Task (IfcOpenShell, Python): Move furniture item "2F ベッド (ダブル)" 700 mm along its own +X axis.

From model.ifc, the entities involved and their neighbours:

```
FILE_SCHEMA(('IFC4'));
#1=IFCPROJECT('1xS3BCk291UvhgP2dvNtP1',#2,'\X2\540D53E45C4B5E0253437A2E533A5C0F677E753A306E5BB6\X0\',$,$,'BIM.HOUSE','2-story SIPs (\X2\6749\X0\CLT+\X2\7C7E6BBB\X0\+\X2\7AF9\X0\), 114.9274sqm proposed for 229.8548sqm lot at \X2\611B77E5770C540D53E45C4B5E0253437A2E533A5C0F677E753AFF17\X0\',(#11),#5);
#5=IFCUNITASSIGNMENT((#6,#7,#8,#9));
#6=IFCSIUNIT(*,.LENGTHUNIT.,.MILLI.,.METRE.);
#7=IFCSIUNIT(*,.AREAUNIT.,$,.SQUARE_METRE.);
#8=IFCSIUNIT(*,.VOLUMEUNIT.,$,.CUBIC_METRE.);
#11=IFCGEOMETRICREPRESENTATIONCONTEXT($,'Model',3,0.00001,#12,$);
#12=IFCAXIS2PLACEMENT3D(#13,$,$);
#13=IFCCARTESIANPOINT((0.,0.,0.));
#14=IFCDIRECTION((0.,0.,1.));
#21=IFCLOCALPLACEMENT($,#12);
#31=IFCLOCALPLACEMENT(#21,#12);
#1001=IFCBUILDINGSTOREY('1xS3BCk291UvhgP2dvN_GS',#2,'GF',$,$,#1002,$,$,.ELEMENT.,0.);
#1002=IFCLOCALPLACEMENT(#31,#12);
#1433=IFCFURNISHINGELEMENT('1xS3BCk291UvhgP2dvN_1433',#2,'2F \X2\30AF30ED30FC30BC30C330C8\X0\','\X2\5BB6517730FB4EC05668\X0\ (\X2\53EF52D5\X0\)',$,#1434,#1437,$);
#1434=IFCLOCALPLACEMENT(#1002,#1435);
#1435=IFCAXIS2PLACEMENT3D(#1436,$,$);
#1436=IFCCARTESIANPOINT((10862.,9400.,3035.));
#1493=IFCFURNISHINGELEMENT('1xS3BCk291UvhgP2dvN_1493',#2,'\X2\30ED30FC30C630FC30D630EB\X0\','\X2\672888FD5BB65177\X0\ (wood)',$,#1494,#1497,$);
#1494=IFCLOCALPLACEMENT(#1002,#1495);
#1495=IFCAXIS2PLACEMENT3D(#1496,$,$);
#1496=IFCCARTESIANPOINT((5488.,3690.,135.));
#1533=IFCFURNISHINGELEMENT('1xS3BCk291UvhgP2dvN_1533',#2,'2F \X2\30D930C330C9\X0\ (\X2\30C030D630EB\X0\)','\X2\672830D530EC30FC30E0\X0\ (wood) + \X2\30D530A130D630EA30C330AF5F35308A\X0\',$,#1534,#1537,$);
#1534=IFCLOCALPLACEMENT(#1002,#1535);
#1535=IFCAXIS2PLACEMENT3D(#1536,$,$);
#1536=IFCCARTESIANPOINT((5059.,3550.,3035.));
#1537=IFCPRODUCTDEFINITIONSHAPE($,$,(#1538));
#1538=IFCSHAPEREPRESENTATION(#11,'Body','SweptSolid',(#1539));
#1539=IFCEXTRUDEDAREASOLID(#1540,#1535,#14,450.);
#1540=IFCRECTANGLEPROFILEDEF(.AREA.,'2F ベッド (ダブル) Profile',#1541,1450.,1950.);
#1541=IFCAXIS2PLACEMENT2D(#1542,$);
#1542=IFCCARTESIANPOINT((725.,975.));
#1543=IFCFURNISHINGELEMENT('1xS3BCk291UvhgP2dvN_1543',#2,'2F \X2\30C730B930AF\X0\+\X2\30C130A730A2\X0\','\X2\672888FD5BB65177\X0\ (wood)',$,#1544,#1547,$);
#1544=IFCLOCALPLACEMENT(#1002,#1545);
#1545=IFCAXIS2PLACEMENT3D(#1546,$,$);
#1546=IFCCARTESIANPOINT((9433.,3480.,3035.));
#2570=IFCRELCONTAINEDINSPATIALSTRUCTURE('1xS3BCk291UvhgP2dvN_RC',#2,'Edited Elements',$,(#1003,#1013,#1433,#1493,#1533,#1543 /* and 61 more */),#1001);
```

```python
import ifcopenshell
import ifcopenshell.api.geometry
import ifcopenshell.util.placement
import ifcopenshell.util.unit

model = ifcopenshell.open("model.ifc")
unit_scale = ifcopenshell.util.unit.calculate_unit_scale(model)

item = model.by_guid("1xS3BCk291UvhgP2dvN_1533")
matrix = ifcopenshell.util.placement.get_local_placement(item.ObjectPlacement)
matrix[:3, 3] += matrix[:3, 0] * 0.7 / unit_scale
ifcopenshell.api.geometry.edit_object_placement(model, product=item, matrix=matrix, is_si=False)

print(ifcopenshell.util.placement.get_local_placement(item.ObjectPlacement).round(3) + 0.0)

model.write("model_rev.ifc")
```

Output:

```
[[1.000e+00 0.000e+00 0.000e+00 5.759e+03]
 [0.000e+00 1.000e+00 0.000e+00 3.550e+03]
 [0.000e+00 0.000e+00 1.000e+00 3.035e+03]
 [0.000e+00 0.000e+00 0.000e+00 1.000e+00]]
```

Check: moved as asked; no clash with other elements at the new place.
